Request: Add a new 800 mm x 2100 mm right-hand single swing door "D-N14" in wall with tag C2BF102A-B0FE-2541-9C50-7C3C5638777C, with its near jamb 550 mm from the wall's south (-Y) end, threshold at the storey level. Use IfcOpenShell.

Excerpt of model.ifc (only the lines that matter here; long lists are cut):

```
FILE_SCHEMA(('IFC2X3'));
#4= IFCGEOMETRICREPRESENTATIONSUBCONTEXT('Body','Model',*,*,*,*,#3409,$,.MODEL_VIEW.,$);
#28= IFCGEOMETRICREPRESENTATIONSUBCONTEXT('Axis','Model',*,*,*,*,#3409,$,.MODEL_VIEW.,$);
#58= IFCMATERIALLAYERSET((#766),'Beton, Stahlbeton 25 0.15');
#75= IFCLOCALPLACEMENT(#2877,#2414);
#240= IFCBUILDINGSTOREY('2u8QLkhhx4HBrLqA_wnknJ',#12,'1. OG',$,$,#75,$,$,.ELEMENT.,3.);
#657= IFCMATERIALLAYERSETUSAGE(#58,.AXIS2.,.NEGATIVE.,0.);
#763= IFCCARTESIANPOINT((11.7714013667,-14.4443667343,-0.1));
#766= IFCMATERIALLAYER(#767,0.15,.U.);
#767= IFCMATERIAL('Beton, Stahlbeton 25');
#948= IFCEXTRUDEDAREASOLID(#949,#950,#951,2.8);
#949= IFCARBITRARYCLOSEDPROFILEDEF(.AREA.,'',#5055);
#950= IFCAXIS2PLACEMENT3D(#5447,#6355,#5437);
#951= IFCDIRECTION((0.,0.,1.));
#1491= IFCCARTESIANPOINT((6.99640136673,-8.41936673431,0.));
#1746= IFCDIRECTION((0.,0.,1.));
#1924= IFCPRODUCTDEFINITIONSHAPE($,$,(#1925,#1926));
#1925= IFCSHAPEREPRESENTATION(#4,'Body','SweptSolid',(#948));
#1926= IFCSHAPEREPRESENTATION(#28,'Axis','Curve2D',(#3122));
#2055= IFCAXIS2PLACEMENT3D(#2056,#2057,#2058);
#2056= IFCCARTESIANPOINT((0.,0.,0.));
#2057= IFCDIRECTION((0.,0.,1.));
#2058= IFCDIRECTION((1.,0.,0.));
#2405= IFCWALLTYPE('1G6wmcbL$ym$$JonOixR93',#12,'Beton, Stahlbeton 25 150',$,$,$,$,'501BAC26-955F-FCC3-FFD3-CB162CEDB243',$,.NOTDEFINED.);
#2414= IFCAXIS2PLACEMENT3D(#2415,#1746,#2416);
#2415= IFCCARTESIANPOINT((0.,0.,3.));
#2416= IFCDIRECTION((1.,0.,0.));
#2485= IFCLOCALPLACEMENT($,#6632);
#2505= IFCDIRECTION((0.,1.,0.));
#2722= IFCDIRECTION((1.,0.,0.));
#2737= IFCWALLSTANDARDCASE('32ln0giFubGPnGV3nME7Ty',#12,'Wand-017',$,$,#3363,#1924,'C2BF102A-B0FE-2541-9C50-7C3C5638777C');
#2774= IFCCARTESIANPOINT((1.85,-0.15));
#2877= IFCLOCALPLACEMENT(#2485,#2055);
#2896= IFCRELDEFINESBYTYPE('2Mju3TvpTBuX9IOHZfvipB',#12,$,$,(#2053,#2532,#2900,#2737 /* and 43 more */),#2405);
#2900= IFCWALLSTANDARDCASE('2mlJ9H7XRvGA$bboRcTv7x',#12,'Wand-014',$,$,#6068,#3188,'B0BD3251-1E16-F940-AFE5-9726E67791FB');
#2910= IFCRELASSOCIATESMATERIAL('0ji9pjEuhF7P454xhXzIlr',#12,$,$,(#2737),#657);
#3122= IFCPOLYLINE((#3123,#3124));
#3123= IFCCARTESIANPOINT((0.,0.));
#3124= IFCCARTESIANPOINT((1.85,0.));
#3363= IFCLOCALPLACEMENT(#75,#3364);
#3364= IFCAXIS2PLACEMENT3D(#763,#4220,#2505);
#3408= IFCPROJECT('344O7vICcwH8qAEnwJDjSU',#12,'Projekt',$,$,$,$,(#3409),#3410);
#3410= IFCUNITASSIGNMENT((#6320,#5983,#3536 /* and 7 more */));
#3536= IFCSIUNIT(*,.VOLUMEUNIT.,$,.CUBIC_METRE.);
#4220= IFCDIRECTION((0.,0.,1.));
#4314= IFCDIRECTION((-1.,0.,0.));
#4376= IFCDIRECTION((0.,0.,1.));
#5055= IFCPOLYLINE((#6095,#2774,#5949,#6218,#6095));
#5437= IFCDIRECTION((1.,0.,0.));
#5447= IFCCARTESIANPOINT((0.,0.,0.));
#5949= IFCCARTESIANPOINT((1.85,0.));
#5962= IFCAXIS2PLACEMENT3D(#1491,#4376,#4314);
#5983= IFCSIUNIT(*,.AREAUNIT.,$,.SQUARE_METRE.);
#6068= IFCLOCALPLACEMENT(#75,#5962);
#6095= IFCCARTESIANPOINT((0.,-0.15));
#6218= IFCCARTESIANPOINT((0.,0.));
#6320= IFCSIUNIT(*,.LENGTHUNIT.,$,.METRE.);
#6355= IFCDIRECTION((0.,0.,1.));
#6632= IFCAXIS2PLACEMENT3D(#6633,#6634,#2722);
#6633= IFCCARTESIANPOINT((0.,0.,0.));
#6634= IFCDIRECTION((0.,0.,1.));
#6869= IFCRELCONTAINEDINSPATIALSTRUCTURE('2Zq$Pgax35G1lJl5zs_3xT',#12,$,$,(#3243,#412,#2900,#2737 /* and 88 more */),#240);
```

```python
import numpy as np
import ifcopenshell
import ifcopenshell.api.feature
import ifcopenshell.api.geometry
import ifcopenshell.api.root
import ifcopenshell.api.spatial
import ifcopenshell.api.type
import ifcopenshell.geom
import ifcopenshell.util.element
import ifcopenshell.util.placement
import ifcopenshell.util.representation
import ifcopenshell.util.shape
import ifcopenshell.util.unit

model = ifcopenshell.open("model.ifc")
unit_scale = ifcopenshell.util.unit.calculate_unit_scale(model)
settings = ifcopenshell.geom.settings()


def volume(element):
    """Net volume in cubic metres, openings subtracted."""
    shape = ifcopenshell.geom.create_shape(settings, element)
    return ifcopenshell.util.shape.get_volume(shape.geometry)


wall = model.by_guid("32ln0giFubGPnGV3nME7Ty")
storey = ifcopenshell.util.element.get_container(wall, ifc_class="IfcBuildingStorey")
context = ifcopenshell.util.representation.get_context(model, "Model", "Body", "MODEL_VIEW")
before = volume(wall)

width, height, from_end, sill = 0.8, 2.1, 0.55, 0.0  # metres

# The wall runs along its own X axis, and the end named is its -X end.
wall_shape = ifcopenshell.geom.create_shape(settings, wall)
x, y, z = ifcopenshell.util.shape.get_vertices(wall_shape.geometry).T
start = x.min() + from_end
face, thickness = float(y.min()), float(y.max() - y.min())
wall_matrix = ifcopenshell.util.placement.get_local_placement(wall.ObjectPlacement)
level = ifcopenshell.util.placement.get_local_placement(storey.ObjectPlacement)[2, 3]


def in_wall(x, y):
    """Placement at x, y metres in the wall's axes, at sill height."""
    matrix = wall_matrix.copy()
    matrix[:, 3] = wall_matrix @ np.array([x / unit_scale, y / unit_scale, 0.0, 1.0])
    matrix[2, 3] = level + sill / unit_scale
    return matrix


# Opening: a box that overshoots both wall faces by 50 mm.
opening = ifcopenshell.api.root.create_entity(model, ifc_class="IfcOpeningElement")
box = ifcopenshell.api.geometry.add_wall_representation(
    model, context=context, length=width, height=height, thickness=thickness + 0.1
)
ifcopenshell.api.geometry.assign_representation(model, product=opening, representation=box)
ifcopenshell.api.geometry.edit_object_placement(model, product=opening, matrix=in_wall(start, face - 0.05), is_si=False)
ifcopenshell.api.feature.add_feature(model, feature=opening, element=wall)

door = ifcopenshell.api.root.create_entity(model, ifc_class="IfcDoor", name="D-N14")
door.OverallWidth, door.OverallHeight = width / unit_scale, height / unit_scale
body = ifcopenshell.api.geometry.add_door_representation(
    model,
    context=context,
    overall_width=door.OverallWidth,
    overall_height=door.OverallHeight,
    operation_type="SINGLE_SWING_RIGHT",
    lining_properties={"LiningDepth": thickness / unit_scale, "ThresholdDepth": thickness / unit_scale},
)
ifcopenshell.api.geometry.assign_representation(model, product=door, representation=body)
ifcopenshell.api.spatial.assign_container(model, products=[door], relating_structure=storey)
fills = ifcopenshell.api.feature.add_filling(model, opening=opening, element=door)
fills.OwnerHistory = door.OwnerHistory  # required in IFC2X3

# IFC2X3 keeps the operation on the door style.
style = ifcopenshell.api.root.create_entity(model, ifc_class="IfcDoorStyle", name="D-N14")
style.OperationType, style.ConstructionType = "SINGLE_SWING_RIGHT", "NOTDEFINED"
style.ParameterTakesPrecedence = style.Sizeable = False
ifcopenshell.api.type.assign_type(model, related_objects=[door], relating_type=style)

# The lining spans the wall, so the door starts at the wall face.
ifcopenshell.api.geometry.edit_object_placement(model, product=door, matrix=in_wall(start, face), is_si=False)

after = volume(wall)

print(f"wall volume {before:.3f} -> {after:.3f} m3")

model.write("model_rev.ifc")
```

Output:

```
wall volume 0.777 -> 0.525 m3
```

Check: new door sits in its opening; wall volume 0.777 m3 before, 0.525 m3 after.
